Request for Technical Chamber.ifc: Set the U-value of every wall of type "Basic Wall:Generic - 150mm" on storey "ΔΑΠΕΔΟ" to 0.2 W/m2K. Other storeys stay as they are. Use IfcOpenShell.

First a look at what the model holds.

```python
import ifcopenshell
import ifcopenshell.util.element

model = ifcopenshell.open("Technical Chamber.ifc")
print(model.schema)
storey = next(s for s in model.by_type("IfcBuildingStorey") if s.Name == "ΔΑΠΕΔΟ")
walls = [e for e in ifcopenshell.util.element.get_decomposition(storey) if e.is_a("IfcWall")]
seen = {}
for e in walls:
    element_type = ifcopenshell.util.element.get_type(e)
    key = (element_type.Name if element_type != e and element_type else None, ifcopenshell.util.element.get_pset(e, "Pset_WallCommon", "ThermalTransmittance"))
    seen[key] = seen.get(key, 0) + 1
for (name, value), count in sorted(seen.items(), key=str):
    print(count, "x", name, "|", value)
```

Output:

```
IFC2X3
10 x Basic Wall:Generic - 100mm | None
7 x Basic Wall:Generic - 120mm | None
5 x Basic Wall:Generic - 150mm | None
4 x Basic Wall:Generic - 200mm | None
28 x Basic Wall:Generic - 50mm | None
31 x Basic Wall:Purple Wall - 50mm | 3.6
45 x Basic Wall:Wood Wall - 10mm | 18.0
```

```python
import ifcopenshell
import ifcopenshell.api.pset
import ifcopenshell.util.element

model = ifcopenshell.open("Technical Chamber.ifc")

storey = next(s for s in model.by_type("IfcBuildingStorey") if s.Name == "ΔΑΠΕΔΟ")
walls = [e for e in ifcopenshell.util.element.get_decomposition(storey) if e.is_a("IfcWall")]

count = 0
for e in walls:
    element_type = ifcopenshell.util.element.get_type(e)
    if element_type in (None, e) or element_type.Name != "Basic Wall:Generic - 150mm":
        continue
    # add_pset returns the element's existing set when there is one.
    pset = ifcopenshell.api.pset.add_pset(model, product=e, name="Pset_WallCommon")
    ifcopenshell.api.pset.edit_pset(model, pset=pset, properties={"ThermalTransmittance": 0.2})
    count += 1

print(count, "walls updated")

model.write("Technical Chamber-out.ifc")
```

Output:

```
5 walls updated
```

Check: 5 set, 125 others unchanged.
